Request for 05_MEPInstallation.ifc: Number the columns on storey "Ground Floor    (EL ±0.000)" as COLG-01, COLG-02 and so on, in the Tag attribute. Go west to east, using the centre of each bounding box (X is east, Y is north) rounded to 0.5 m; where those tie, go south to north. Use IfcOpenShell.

First a look at what the model holds.

```python
import ifcopenshell
import ifcopenshell.util.element
import ifcopenshell.util.placement

model = ifcopenshell.open("05_MEPInstallation.ifc")
print(model.schema)
storey = next(s for s in model.by_type("IfcBuildingStorey") if s.Name == "Ground Floor    (EL ±0.000)")
columns = [e for e in ifcopenshell.util.element.get_decomposition(storey) if e.is_a("IfcColumn")]
for e in sorted(columns, key=lambda e: e.id()):
    origin = ifcopenshell.util.placement.get_local_placement(e.ObjectPlacement)[:3, 3]
    print(e.id(), e.Tag, e.Name, origin.round(2) + 0.0, sep=" | ")
```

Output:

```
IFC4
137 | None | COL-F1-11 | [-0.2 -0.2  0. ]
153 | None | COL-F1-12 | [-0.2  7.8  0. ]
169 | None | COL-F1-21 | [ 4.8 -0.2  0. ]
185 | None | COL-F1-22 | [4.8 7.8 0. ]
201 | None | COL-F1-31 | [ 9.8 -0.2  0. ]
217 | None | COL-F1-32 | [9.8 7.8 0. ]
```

```python
import ifcopenshell
import ifcopenshell.geom
import ifcopenshell.util.element
import ifcopenshell.util.shape

model = ifcopenshell.open("05_MEPInstallation.ifc")
settings = ifcopenshell.geom.settings()
settings.set("use-world-coords", True)


def centre(element):
    shape = ifcopenshell.geom.create_shape(settings, element)
    return ifcopenshell.util.shape.get_bbox_centroid(shape.geometry)


storey = next(s for s in model.by_type("IfcBuildingStorey") if s.Name == "Ground Floor    (EL ±0.000)")
columns = [e for e in ifcopenshell.util.element.get_decomposition(storey) if e.is_a("IfcColumn")]

# Insertion points can sit at a corner or the storey origin, so sort by the geometry (in metres).
centres = {e: centre(e) for e in columns}
columns.sort(key=lambda e: (round(centres[e][0] / 0.5), centres[e][1]))

for i, e in enumerate(columns, start=1):
    number = f"COLG-{i:02d}"
    e.Tag = number
    print(e.id(), number)

model.write("05_MEPInstallation-out.ifc")
```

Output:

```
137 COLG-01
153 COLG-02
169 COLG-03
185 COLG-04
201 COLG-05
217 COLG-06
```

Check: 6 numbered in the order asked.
